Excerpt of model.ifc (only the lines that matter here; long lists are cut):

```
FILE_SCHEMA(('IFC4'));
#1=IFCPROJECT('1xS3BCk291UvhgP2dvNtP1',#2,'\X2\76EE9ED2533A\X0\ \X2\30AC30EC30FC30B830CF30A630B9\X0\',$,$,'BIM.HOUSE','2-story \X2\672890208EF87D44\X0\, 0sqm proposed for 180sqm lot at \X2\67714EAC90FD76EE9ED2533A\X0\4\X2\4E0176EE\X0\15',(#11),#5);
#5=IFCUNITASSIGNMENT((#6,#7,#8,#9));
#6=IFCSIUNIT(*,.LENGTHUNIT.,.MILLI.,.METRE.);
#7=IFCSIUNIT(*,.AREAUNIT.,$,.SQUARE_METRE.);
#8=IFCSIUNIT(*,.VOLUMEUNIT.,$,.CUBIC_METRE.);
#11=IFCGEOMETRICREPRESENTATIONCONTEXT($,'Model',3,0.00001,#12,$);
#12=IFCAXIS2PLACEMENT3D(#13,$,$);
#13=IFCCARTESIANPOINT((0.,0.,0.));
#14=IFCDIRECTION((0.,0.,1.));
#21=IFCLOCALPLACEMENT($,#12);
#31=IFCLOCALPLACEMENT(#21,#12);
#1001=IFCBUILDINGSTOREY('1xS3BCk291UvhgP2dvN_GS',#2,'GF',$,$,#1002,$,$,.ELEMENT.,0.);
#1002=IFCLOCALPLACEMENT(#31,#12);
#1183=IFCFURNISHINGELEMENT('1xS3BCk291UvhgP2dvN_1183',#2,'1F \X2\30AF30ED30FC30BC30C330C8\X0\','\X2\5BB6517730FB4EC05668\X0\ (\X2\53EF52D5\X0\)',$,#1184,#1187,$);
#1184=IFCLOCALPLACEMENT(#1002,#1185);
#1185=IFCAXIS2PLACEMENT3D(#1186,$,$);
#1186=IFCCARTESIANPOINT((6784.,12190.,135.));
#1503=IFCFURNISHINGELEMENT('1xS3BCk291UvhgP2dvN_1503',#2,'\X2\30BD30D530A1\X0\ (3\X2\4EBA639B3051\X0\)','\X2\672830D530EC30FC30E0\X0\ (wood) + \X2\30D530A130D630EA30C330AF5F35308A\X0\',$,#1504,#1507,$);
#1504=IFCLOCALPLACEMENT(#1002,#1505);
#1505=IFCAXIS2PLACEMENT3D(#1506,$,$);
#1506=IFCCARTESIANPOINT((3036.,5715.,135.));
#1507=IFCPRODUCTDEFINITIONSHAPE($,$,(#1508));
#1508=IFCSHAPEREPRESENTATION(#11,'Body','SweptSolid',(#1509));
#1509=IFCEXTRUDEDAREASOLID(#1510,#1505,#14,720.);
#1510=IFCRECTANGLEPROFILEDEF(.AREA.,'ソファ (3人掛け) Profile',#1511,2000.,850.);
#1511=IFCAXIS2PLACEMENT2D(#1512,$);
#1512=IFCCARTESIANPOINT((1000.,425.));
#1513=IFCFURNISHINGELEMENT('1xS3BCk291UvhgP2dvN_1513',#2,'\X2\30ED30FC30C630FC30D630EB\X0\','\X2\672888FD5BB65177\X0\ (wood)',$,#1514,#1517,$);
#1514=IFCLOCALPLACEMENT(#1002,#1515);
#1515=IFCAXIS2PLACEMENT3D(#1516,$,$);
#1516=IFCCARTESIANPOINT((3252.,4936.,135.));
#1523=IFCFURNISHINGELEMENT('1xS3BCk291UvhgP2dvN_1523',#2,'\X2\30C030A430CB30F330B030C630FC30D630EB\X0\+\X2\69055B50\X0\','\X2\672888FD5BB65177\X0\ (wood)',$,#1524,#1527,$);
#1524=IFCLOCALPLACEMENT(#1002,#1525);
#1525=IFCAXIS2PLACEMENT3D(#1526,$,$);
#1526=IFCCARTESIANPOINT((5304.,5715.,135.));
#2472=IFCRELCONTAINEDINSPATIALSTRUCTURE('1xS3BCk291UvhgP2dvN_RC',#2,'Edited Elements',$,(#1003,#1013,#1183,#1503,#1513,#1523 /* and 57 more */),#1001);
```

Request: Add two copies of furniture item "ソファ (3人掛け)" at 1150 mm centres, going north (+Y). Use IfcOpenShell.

```python
import numpy as np
import ifcopenshell
import ifcopenshell.api.geometry
import ifcopenshell.api.root
import ifcopenshell.util.element
import ifcopenshell.util.placement

model = ifcopenshell.open("model.ifc")


def reuse_history(source, copy):
    """copy_class also copies each property set's owner history, people and application; keep the originals."""
    for rel in copy.IsDefinedBy:
        if rel.is_a("IfcRelDefinesByProperties") and (history := rel.RelatingPropertyDefinition.OwnerHistory):
            rel.RelatingPropertyDefinition.OwnerHistory = source.OwnerHistory
            ifcopenshell.util.element.remove_deep2(model, history)


source = model.by_id(1503)
base = ifcopenshell.util.placement.get_local_placement(source.ObjectPlacement)
step = np.array([0.0, 1.0, 0.0]) * 1150.0

for i in range(1, 3):
    copy = ifcopenshell.api.root.copy_class(model, product=source)
    copy.Representation = ifcopenshell.util.element.copy_deep(
        model, source.Representation, exclude=["IfcGeometricRepresentationContext", "IfcRepresentationMap"]
    )
    reuse_history(source, copy)
    matrix = base.copy()
    matrix[:3, 3] += i * step
    print("added at", matrix[:3, 3].round(3) + 0.0)
    ifcopenshell.api.geometry.edit_object_placement(model, product=copy, matrix=matrix, is_si=False)

model.write("model_updated.ifc")
```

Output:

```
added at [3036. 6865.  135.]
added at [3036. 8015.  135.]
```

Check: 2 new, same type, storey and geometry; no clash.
